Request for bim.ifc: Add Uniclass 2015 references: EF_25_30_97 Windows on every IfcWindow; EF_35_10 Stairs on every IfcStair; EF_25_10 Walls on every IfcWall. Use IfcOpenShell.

First a look at what the model holds.

```python
import ifcopenshell

model = ifcopenshell.open("bim.ifc")
print(model.schema)
print("classifications:", [c.Name for c in model.by_type("IfcClassification")])
for ifc_class in ("IfcDoor", "IfcRoof", "IfcStair", "IfcWall", "IfcWindow"):
    print(ifc_class, len(model.by_type(ifc_class)))
```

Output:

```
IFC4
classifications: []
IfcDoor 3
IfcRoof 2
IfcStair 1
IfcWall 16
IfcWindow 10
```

```python
import ifcopenshell
import ifcopenshell.api.classification

model = ifcopenshell.open("bim.ifc")

system = ifcopenshell.api.classification.add_classification(model, classification="Uniclass 2015")

codes = {
    "IfcWindow": ("EF_25_30_97", "Windows"),
    "IfcStair": ("EF_35_10", "Stairs"),
    "IfcWall": ("EF_25_10", "Walls"),
}
for ifc_class, (code, name) in codes.items():
    products = model.by_type(ifc_class)
    ifcopenshell.api.classification.add_reference(
        model, products=products, classification=system, identification=code, name=name
    )
    print(code, len(products))

model.write("bim_edited.ifc")
```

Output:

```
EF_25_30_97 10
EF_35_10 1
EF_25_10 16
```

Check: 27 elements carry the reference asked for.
